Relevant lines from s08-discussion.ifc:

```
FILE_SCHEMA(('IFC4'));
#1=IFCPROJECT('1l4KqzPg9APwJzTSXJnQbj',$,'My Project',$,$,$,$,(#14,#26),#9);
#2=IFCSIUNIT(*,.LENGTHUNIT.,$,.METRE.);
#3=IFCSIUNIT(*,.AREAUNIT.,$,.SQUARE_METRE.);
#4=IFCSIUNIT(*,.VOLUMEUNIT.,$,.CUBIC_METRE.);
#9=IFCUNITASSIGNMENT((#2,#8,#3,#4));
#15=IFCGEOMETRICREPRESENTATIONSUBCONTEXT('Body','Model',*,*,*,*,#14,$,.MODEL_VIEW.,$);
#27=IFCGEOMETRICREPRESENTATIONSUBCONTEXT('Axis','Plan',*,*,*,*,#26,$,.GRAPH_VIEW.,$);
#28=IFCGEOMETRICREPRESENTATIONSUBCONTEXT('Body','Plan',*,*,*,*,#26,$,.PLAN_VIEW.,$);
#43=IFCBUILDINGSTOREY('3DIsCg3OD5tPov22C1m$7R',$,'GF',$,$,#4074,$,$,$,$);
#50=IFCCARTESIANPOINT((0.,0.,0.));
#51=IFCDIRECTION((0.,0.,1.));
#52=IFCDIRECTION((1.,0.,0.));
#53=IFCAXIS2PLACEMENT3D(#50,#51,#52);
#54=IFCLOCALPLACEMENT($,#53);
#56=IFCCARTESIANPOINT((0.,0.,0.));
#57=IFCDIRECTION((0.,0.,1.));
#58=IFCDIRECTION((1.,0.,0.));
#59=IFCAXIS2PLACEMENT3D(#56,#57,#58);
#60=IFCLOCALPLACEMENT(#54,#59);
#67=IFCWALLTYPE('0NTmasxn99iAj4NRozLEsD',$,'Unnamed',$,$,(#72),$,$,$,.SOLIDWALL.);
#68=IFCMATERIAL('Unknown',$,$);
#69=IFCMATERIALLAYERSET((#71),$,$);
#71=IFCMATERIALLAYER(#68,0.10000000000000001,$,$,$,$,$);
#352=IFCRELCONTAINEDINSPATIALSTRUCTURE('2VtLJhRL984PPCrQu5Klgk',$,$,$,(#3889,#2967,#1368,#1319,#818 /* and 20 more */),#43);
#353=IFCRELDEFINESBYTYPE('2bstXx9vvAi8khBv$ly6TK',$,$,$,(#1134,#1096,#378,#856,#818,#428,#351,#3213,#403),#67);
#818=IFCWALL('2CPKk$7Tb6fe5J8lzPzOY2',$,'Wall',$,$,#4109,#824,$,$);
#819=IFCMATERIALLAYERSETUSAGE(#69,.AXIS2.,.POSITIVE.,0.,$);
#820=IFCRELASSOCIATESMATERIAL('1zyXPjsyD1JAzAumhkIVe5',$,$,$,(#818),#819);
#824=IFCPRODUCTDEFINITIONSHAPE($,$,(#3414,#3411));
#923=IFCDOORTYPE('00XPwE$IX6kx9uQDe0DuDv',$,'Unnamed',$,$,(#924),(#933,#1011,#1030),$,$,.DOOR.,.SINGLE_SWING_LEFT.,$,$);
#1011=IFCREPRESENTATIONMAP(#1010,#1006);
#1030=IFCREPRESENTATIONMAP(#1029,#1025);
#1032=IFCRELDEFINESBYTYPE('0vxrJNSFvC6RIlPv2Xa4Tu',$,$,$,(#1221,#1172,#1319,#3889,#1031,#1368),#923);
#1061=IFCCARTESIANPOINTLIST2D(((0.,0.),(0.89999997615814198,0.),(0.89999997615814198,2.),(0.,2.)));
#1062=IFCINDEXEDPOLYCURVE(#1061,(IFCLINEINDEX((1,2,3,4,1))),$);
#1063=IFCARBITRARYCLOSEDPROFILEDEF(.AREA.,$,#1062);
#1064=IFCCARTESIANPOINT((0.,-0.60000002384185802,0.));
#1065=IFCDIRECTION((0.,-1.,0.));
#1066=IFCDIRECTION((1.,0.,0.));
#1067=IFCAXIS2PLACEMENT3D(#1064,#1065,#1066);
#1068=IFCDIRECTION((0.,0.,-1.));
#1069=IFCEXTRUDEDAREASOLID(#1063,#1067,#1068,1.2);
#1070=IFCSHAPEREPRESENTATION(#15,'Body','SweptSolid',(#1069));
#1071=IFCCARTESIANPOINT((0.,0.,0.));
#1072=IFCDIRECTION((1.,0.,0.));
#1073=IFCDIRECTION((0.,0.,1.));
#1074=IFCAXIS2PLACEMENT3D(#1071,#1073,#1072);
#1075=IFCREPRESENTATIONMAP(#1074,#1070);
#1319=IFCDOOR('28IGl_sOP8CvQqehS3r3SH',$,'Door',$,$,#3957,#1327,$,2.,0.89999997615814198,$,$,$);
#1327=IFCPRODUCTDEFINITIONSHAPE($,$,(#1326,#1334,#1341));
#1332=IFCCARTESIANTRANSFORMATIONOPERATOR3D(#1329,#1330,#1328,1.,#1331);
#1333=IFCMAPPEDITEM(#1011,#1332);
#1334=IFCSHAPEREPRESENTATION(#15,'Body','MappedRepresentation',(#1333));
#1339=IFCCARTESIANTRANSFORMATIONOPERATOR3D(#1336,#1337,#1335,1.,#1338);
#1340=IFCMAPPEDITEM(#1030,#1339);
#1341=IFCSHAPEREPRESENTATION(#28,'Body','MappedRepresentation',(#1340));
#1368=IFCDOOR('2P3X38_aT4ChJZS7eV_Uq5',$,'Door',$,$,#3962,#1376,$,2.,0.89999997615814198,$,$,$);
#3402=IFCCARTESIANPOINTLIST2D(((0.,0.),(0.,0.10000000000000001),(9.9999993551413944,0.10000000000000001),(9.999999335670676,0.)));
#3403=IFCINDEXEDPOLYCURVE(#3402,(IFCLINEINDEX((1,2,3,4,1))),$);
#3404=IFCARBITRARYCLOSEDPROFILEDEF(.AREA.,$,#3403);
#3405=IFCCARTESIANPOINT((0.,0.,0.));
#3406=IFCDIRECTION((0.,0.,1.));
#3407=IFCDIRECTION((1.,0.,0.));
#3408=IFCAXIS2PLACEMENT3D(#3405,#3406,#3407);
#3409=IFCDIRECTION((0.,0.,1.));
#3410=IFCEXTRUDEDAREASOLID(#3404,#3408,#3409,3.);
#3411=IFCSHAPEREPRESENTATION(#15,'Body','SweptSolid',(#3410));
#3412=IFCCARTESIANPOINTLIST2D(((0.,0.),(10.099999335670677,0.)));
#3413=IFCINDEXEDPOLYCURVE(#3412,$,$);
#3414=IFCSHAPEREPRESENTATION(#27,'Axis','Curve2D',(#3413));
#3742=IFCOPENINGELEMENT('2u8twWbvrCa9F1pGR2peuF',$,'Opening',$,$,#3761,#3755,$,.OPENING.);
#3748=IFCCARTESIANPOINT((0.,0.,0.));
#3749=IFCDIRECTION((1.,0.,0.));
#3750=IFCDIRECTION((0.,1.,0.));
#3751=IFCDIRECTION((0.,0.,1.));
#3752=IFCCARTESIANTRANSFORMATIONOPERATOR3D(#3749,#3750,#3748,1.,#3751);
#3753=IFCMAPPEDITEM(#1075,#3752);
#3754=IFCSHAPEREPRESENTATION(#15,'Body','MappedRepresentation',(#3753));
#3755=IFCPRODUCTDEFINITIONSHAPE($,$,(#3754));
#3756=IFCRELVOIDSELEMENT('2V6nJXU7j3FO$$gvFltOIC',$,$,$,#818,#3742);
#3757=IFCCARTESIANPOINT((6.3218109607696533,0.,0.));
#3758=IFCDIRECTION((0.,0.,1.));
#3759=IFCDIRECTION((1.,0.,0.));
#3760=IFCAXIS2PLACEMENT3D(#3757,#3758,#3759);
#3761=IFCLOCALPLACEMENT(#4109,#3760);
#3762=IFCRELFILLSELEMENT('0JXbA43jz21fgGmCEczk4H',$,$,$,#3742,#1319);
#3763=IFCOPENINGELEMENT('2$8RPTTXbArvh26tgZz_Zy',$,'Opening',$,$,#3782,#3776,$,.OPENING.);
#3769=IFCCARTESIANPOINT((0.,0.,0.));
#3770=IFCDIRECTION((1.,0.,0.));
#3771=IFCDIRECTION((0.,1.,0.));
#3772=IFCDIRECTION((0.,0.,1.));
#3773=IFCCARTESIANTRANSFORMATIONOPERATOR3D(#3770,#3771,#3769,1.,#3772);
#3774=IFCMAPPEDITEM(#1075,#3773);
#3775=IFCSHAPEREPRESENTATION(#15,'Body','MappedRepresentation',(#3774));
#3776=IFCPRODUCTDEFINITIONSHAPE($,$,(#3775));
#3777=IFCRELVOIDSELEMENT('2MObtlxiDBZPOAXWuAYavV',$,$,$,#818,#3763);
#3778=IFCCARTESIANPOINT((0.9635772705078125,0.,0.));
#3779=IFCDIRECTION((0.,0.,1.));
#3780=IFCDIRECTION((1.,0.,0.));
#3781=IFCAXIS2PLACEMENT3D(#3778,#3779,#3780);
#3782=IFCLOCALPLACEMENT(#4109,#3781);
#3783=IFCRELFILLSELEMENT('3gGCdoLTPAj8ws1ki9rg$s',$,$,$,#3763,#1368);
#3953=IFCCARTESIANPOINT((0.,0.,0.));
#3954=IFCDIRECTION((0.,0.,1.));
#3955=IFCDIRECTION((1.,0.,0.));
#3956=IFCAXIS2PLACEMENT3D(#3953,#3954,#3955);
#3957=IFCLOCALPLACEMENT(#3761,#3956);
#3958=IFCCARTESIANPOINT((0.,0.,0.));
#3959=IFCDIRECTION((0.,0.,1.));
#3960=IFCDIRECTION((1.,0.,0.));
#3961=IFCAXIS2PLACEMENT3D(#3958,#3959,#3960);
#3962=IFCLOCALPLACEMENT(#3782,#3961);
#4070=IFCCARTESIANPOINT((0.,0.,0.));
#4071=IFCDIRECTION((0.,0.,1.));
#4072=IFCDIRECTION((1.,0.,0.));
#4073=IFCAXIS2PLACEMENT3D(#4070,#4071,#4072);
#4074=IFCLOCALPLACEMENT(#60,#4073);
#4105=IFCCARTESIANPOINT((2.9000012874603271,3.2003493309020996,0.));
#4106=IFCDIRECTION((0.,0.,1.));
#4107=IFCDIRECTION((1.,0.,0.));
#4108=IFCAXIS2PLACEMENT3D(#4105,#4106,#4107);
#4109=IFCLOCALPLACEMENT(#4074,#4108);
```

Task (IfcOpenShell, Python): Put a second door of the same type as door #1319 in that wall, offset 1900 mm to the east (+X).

```python
import ifcopenshell
import ifcopenshell.api.feature
import ifcopenshell.api.geometry
import ifcopenshell.api.root
import ifcopenshell.geom
import ifcopenshell.util.element
import ifcopenshell.util.placement
import ifcopenshell.util.shape

model = ifcopenshell.open("s08-discussion.ifc")
settings = ifcopenshell.geom.settings()


def volume(element):
    """Net volume in cubic metres, openings subtracted."""
    shape = ifcopenshell.geom.create_shape(settings, element)
    return ifcopenshell.util.shape.get_volume(shape.geometry)


door = model.by_id(1319)
opening = door.FillsVoids[0].RelatingOpeningElement
wall = opening.VoidsElements[0].RelatingBuildingElement
before = volume(wall)
shift = ifcopenshell.util.placement.get_local_placement(wall.ObjectPlacement)[:3, 0] * 1.9

# copy_class copies the void relationship, type, container and properties, but no geometry.
new_opening = ifcopenshell.api.root.copy_class(model, product=opening)
new_opening.Representation = ifcopenshell.util.element.copy_deep(
    model, opening.Representation, exclude=["IfcGeometricRepresentationContext", "IfcRepresentationMap"]
)
new_door = ifcopenshell.api.root.copy_class(model, product=door)
new_door.Representation = ifcopenshell.util.element.copy_deep(
    model, door.Representation, exclude=["IfcGeometricRepresentationContext", "IfcRepresentationMap"]
)
ifcopenshell.api.feature.add_filling(model, opening=new_opening, element=new_door)

for old, new in ((opening, new_opening), (door, new_door)):
    matrix = ifcopenshell.util.placement.get_local_placement(old.ObjectPlacement)
    matrix[:3, 3] += shift
    ifcopenshell.api.geometry.edit_object_placement(model, product=new, matrix=matrix, is_si=False)

after = volume(wall)

print(f"wall volume {before:.3f} -> {after:.3f} m3")

model.write("s08-discussion_edited.ifc")
```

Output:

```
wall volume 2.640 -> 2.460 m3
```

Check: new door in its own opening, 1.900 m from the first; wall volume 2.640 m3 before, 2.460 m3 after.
